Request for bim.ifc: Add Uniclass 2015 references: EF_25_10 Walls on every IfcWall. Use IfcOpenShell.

First a look at what the model holds.

```python
import ifcopenshell

model = ifcopenshell.open("bim.ifc")
print(model.schema)
print("classifications:", [c.Name for c in model.by_type("IfcClassification")])
for ifc_class in ("IfcDoor", "IfcRoof", "IfcStair", "IfcWall", "IfcWindow"):
    print(ifc_class, len(model.by_type(ifc_class)))
```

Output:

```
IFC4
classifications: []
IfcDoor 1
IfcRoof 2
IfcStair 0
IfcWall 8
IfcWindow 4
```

```python
import ifcopenshell
import ifcopenshell.api.classification

model = ifcopenshell.open("bim.ifc")

system = ifcopenshell.api.classification.add_classification(model, classification="Uniclass 2015")

codes = {
    "IfcWall": ("EF_25_10", "Walls"),
}
for ifc_class, (code, name) in codes.items():
    products = model.by_type(ifc_class)
    ifcopenshell.api.classification.add_reference(
        model, products=products, classification=system, identification=code, name=name
    )
    print(code, len(products))

model.write("bim_updated.ifc")
```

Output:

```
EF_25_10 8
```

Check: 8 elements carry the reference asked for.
